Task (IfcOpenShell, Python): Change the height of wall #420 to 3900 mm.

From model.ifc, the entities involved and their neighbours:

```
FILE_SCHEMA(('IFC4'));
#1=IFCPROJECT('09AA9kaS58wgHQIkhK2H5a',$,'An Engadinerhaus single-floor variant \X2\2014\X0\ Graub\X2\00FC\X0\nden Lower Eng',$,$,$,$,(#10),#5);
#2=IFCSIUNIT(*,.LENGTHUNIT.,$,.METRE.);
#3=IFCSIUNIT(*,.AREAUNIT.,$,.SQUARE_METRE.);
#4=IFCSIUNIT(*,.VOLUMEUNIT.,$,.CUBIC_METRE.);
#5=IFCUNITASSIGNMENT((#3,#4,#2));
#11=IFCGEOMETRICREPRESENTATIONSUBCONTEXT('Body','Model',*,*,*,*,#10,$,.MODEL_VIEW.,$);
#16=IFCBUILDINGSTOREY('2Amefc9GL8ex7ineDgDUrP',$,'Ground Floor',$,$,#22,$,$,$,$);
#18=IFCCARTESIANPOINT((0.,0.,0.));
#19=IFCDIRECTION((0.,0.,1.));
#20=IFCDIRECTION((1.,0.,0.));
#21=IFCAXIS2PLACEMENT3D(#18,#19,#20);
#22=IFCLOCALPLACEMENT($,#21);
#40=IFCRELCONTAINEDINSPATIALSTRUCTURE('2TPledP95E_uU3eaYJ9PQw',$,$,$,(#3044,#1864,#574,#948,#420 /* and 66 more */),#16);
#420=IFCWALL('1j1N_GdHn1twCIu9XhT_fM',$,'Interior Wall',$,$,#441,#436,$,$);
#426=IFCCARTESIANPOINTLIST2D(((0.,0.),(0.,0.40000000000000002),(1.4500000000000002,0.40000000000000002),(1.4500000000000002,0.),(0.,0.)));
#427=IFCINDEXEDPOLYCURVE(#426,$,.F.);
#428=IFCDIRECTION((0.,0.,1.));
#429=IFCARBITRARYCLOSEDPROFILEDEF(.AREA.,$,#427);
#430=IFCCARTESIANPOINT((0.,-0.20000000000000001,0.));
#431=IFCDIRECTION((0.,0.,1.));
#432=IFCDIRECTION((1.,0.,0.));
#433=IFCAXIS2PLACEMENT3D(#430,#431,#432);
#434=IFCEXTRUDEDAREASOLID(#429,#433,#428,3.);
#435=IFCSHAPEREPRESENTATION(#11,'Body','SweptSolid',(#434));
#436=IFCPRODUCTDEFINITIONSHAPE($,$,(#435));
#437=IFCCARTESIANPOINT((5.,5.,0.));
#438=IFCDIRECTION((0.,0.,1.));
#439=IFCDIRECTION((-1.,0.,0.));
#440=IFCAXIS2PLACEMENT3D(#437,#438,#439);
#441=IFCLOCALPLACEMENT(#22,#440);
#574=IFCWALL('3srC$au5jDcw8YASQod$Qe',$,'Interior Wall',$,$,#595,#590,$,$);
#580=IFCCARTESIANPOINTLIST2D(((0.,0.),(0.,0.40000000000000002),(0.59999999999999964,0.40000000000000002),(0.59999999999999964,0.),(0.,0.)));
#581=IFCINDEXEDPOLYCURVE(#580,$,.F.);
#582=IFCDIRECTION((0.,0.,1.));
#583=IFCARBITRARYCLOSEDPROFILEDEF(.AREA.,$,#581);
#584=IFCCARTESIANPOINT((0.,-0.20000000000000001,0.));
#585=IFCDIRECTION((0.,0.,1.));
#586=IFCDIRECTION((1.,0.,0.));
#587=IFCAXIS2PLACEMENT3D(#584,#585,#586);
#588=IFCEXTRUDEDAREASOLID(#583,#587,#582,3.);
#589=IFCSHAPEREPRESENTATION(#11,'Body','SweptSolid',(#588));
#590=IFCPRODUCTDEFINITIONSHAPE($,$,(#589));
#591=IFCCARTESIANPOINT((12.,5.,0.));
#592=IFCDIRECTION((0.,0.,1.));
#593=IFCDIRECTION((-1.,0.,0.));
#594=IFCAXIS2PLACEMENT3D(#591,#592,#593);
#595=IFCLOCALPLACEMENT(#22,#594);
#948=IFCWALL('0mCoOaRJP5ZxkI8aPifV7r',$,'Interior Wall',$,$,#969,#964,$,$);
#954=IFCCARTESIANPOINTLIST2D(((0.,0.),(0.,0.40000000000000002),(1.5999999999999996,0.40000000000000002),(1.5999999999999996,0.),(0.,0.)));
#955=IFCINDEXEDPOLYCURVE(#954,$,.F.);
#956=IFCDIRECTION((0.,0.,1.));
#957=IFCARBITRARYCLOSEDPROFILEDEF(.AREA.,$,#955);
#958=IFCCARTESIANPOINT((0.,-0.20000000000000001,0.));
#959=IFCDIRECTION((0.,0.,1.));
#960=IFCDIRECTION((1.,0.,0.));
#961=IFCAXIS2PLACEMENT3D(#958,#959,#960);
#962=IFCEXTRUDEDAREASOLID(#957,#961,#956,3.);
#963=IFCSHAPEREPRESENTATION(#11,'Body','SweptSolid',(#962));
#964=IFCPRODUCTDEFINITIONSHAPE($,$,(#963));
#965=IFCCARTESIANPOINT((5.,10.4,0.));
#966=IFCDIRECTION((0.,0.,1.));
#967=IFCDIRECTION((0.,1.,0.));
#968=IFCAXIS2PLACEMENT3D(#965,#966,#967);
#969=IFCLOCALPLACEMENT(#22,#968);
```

```python
import ifcopenshell
import ifcopenshell.geom
import ifcopenshell.util.representation
import ifcopenshell.util.shape
import ifcopenshell.util.unit

model = ifcopenshell.open("model.ifc")
unit_scale = ifcopenshell.util.unit.calculate_unit_scale(model)
settings = ifcopenshell.geom.settings()


def volume(element):
    """Net volume in cubic metres, openings subtracted."""
    shape = ifcopenshell.geom.create_shape(settings, element)
    return ifcopenshell.util.shape.get_volume(shape.geometry)


wall = model.by_guid("1j1N_GdHn1twCIu9XhT_fM")
before = volume(wall)

body = ifcopenshell.util.representation.get_representation(wall, "Model", "Body")
solid = body.Items[0]
old_height = solid.Depth
solid.Depth = 3.9 / unit_scale
after = volume(wall)

print(f"height {old_height:g} -> {solid.Depth:g}, volume {before:.3f} -> {after:.3f} m3")

model.write("model_edited.ifc")
```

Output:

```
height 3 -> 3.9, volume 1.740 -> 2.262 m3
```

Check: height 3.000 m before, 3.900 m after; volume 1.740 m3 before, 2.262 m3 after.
